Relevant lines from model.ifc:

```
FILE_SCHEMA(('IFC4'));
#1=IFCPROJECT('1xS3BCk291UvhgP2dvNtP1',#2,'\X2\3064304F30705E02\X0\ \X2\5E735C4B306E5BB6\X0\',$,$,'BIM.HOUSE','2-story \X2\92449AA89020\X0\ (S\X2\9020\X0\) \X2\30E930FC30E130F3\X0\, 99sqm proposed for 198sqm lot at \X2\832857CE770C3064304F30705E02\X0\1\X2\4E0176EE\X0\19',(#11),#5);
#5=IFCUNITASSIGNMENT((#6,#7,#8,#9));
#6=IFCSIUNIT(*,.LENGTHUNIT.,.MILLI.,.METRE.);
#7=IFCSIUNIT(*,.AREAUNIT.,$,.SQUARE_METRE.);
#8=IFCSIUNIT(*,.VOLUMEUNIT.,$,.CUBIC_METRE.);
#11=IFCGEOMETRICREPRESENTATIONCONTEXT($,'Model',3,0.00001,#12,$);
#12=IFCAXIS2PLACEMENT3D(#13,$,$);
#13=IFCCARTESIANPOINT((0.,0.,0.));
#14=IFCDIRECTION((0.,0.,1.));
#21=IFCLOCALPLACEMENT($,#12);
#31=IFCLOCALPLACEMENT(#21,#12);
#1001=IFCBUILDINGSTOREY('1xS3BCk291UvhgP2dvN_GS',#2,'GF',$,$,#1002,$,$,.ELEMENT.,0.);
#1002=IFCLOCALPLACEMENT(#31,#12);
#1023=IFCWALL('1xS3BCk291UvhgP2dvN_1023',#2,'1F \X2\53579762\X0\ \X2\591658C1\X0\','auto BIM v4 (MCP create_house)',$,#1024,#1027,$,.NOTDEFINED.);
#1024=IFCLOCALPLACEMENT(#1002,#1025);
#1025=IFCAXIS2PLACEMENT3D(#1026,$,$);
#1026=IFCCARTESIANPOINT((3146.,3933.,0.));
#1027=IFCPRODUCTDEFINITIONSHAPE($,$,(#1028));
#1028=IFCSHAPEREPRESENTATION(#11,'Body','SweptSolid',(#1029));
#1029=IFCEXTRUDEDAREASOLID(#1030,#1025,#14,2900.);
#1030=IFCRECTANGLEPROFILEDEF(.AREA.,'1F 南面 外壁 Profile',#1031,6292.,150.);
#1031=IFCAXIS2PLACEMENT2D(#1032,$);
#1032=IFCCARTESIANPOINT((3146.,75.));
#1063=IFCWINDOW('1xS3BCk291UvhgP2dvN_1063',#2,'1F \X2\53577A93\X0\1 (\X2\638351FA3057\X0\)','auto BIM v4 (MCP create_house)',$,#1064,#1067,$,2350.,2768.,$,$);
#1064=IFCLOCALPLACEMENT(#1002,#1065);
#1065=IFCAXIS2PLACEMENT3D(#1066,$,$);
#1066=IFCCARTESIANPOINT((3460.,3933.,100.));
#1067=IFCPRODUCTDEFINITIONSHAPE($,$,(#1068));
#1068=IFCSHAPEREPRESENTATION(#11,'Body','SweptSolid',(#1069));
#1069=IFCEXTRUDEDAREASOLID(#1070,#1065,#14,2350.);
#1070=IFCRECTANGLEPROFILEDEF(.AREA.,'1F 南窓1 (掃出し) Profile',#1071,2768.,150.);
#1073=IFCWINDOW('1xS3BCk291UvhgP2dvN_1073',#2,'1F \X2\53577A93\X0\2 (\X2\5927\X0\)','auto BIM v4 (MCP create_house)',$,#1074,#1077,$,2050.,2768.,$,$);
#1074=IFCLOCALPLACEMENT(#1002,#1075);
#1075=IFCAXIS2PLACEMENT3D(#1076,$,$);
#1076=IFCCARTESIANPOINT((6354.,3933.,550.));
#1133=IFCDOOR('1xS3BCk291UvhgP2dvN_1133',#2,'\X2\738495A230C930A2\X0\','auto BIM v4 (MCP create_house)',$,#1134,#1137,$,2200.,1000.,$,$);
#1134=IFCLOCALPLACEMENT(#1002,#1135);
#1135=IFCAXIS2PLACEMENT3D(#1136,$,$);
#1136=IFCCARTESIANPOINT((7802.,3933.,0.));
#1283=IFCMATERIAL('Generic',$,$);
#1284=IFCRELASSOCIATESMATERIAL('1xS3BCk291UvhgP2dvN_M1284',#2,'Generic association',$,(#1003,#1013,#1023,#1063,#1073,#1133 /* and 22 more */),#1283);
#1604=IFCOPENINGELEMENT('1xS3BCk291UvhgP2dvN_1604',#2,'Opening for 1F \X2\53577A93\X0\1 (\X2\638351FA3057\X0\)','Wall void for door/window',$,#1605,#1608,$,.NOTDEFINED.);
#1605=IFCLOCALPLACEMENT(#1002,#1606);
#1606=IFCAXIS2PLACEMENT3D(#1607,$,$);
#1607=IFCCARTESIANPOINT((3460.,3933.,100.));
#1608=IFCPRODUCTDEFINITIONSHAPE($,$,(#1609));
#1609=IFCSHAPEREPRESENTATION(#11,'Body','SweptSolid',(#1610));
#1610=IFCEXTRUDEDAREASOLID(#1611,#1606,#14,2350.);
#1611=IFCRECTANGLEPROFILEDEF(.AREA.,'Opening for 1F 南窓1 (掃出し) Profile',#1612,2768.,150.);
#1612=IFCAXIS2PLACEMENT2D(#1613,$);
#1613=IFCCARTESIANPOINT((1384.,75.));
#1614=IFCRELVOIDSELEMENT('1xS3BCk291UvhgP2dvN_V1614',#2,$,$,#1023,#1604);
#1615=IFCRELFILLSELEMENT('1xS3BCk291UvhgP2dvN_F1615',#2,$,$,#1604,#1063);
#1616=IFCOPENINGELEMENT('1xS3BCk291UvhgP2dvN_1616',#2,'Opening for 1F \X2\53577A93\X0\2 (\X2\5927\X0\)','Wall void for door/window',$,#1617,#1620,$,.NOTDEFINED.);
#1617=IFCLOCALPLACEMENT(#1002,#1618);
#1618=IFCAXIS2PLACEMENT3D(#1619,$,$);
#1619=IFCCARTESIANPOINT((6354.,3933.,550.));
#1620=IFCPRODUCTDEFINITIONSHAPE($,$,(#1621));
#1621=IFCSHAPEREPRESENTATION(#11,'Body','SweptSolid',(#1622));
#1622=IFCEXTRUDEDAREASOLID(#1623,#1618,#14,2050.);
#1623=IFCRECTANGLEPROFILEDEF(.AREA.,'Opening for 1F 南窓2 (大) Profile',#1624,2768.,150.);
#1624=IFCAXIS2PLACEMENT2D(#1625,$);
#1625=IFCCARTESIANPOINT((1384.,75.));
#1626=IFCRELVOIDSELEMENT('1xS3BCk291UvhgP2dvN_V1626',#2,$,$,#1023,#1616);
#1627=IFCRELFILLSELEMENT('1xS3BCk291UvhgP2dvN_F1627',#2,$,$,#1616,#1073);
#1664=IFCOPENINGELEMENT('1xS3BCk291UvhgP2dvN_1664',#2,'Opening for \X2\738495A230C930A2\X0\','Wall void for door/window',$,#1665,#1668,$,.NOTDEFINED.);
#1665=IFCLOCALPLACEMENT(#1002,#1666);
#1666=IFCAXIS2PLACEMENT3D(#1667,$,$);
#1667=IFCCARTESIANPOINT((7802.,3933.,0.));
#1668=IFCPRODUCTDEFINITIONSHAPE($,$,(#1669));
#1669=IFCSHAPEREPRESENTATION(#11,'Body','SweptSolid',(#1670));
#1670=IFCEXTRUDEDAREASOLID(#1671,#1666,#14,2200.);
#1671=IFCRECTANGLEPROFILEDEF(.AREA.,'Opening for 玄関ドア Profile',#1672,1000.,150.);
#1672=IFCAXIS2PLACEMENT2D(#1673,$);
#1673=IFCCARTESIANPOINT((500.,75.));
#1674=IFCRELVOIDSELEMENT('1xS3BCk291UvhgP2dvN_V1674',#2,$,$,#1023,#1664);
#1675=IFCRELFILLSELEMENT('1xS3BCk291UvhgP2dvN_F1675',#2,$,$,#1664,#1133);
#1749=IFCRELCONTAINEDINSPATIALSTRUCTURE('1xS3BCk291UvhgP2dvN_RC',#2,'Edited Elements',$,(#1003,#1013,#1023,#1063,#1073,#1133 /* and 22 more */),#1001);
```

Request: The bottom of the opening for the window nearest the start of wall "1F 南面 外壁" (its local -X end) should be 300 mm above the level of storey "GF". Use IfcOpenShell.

```python
import numpy as np
import ifcopenshell
import ifcopenshell.api.geometry
import ifcopenshell.geom
import ifcopenshell.util.element
import ifcopenshell.util.placement
import ifcopenshell.util.shape
import ifcopenshell.util.unit

model = ifcopenshell.open("model.ifc")
unit_scale = ifcopenshell.util.unit.calculate_unit_scale(model)

window = model.by_guid("1xS3BCk291UvhgP2dvN_1063")
opening = window.FillsVoids[0].RelatingOpeningElement
storey = ifcopenshell.util.element.get_container(window, ifc_class="IfcBuildingStorey")
level = ifcopenshell.util.placement.get_local_placement(storey.ObjectPlacement)[2, 3]

# The opening's origin need not be at the sill, so measure its lowest point.
shape = ifcopenshell.geom.create_shape(ifcopenshell.geom.settings(), opening)
bottom = ifcopenshell.util.shape.get_shape_bottom_elevation(shape, shape.geometry) / unit_scale
dz = level + 0.3 / unit_scale - bottom

shift = np.array([0.0, 0.0, dz])
# The window is not placed relative to its opening, so move both.
for product in (opening, window):
    matrix = ifcopenshell.util.placement.get_local_placement(product.ObjectPlacement)
    matrix[:3, 3] += shift
    ifcopenshell.api.geometry.edit_object_placement(model, product=product, matrix=matrix, is_si=False)

print(f"moved by {dz * unit_scale:+.3f} m")

model.write("model_v2.ifc")
```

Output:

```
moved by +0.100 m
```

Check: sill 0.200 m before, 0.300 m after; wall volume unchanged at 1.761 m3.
